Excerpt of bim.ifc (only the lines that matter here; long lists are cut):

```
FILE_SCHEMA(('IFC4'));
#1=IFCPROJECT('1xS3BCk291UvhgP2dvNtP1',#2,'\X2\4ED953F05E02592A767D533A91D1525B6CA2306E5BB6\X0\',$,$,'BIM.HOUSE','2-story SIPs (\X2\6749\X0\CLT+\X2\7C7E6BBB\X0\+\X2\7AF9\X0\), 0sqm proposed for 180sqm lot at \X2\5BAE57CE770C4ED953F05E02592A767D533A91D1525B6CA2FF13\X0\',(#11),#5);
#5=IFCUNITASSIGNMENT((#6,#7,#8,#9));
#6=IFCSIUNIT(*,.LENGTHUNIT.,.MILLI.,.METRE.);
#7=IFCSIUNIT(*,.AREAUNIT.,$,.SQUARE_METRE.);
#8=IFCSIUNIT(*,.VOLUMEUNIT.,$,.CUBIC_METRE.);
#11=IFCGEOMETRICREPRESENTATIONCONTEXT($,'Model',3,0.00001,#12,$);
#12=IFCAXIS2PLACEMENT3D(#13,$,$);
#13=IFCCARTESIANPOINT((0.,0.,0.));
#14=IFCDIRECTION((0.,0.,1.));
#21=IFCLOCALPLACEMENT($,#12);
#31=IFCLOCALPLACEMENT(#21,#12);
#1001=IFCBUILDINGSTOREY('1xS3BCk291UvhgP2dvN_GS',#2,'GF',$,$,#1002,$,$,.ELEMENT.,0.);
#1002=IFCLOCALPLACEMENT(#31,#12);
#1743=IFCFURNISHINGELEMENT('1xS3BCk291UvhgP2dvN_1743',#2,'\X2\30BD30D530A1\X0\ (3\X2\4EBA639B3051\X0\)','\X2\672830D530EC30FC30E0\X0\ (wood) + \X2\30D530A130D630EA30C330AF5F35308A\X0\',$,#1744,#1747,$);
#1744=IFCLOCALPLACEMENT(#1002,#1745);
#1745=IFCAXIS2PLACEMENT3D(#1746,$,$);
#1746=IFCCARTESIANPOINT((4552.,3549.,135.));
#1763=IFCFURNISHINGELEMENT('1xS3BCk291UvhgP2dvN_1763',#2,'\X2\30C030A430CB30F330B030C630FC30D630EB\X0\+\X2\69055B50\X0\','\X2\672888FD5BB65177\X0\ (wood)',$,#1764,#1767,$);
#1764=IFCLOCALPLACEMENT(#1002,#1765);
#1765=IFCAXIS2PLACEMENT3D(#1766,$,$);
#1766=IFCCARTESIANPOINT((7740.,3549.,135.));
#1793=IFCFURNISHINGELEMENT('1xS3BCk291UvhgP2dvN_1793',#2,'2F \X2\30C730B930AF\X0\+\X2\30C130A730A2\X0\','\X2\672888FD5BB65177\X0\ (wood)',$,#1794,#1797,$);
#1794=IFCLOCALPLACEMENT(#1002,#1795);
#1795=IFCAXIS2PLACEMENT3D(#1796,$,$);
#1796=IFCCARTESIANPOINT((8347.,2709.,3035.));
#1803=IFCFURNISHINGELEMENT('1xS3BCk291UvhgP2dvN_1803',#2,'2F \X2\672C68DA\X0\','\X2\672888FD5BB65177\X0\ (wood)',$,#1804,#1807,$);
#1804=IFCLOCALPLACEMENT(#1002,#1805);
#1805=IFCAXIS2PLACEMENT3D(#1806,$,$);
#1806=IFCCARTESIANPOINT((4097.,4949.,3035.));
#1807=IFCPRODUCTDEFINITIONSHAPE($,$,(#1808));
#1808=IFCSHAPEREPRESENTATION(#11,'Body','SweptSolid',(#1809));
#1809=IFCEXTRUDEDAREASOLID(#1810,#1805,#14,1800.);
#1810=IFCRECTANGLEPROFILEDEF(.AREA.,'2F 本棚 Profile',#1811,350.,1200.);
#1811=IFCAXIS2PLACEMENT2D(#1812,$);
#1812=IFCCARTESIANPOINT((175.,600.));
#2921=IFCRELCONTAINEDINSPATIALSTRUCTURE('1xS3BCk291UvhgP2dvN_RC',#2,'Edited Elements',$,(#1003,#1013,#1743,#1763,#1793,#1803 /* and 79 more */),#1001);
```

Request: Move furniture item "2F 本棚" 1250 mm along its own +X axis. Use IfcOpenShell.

```python
import ifcopenshell
import ifcopenshell.api.geometry
import ifcopenshell.util.placement
import ifcopenshell.util.unit

model = ifcopenshell.open("bim.ifc")
unit_scale = ifcopenshell.util.unit.calculate_unit_scale(model)

item = model.by_guid("1xS3BCk291UvhgP2dvN_1803")
matrix = ifcopenshell.util.placement.get_local_placement(item.ObjectPlacement)
matrix[:3, 3] += matrix[:3, 0] * 1.25 / unit_scale
ifcopenshell.api.geometry.edit_object_placement(model, product=item, matrix=matrix, is_si=False)

print(ifcopenshell.util.placement.get_local_placement(item.ObjectPlacement).round(3) + 0.0)

model.write("bim_v2.ifc")
```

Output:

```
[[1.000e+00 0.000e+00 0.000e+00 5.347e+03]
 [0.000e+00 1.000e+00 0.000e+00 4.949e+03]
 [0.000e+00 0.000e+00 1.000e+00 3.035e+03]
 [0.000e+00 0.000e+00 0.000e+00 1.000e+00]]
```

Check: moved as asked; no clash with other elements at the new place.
